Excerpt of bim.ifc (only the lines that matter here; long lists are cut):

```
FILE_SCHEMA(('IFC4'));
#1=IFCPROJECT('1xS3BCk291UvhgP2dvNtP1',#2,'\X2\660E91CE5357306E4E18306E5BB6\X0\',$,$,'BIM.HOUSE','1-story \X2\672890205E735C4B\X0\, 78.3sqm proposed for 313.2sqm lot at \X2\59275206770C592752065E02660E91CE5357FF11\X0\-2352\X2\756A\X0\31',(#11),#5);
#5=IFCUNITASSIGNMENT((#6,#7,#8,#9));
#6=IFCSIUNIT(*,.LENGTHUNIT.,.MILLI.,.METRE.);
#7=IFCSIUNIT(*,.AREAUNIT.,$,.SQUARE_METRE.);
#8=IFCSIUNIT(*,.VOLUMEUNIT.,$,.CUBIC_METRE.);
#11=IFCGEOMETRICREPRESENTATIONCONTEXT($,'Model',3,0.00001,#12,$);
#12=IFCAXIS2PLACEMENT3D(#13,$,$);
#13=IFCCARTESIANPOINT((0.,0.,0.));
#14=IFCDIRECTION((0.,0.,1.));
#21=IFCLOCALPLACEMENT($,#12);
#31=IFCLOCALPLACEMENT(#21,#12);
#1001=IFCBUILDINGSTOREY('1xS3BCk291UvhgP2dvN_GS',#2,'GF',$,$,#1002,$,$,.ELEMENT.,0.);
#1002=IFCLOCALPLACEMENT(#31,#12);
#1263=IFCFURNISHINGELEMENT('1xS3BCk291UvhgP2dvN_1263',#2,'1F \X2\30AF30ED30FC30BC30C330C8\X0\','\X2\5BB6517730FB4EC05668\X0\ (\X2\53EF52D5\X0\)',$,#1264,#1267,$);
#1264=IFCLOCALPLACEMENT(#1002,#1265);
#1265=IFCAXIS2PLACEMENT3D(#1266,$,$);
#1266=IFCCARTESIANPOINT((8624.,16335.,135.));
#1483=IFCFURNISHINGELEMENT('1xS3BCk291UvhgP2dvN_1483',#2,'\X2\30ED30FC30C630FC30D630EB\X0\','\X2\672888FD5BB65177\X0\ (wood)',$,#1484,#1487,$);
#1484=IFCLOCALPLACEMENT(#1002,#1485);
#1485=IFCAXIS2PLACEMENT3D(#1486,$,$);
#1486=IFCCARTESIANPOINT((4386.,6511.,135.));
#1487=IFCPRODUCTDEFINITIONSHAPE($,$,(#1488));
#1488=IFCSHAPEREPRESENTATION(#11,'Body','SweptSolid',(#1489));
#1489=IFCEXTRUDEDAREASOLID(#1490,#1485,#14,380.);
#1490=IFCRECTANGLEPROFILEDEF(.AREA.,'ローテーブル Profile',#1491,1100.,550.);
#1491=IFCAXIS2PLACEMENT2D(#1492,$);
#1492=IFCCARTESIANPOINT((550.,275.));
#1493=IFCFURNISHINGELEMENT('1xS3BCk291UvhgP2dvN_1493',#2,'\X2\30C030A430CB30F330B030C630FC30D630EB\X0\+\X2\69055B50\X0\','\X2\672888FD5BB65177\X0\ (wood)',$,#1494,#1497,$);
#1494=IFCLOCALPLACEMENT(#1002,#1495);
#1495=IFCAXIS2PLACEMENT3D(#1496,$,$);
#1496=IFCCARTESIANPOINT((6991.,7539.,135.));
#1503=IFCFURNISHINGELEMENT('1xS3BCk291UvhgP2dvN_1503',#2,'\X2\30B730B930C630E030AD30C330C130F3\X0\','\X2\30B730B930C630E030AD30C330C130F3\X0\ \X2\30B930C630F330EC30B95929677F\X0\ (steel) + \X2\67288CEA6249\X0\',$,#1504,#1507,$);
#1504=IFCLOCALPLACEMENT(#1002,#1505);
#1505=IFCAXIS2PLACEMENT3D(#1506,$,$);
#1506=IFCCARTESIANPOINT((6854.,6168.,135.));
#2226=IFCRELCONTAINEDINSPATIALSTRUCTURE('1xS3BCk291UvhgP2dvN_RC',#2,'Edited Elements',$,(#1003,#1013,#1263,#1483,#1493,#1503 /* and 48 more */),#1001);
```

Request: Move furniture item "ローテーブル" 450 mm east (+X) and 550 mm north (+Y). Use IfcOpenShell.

```python
import ifcopenshell
import ifcopenshell.api.geometry
import ifcopenshell.util.placement
import ifcopenshell.util.unit

model = ifcopenshell.open("bim.ifc")
unit_scale = ifcopenshell.util.unit.calculate_unit_scale(model)

item = model.by_guid("1xS3BCk291UvhgP2dvN_1483")
matrix = ifcopenshell.util.placement.get_local_placement(item.ObjectPlacement)
matrix[0, 3] += 0.45 / unit_scale
matrix[1, 3] += 0.55 / unit_scale
ifcopenshell.api.geometry.edit_object_placement(model, product=item, matrix=matrix, is_si=False)

print(ifcopenshell.util.placement.get_local_placement(item.ObjectPlacement).round(3) + 0.0)

model.write("bim_updated.ifc")
```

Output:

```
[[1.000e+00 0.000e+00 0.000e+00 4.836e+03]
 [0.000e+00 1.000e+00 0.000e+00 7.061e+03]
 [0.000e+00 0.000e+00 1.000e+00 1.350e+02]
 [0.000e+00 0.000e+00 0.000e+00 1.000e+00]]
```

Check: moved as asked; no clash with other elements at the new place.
